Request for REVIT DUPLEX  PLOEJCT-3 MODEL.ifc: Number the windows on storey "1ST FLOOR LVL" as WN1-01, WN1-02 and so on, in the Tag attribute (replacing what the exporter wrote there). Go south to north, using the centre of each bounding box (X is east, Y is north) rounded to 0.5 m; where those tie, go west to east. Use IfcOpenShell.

First a look at what the model holds.

```python
import ifcopenshell
import ifcopenshell.util.element
import ifcopenshell.util.placement

model = ifcopenshell.open("REVIT DUPLEX  PLOEJCT-3 MODEL.ifc")
print(model.schema)
storey = next(s for s in model.by_type("IfcBuildingStorey") if s.Name == "1ST FLOOR LVL")
windows = [e for e in ifcopenshell.util.element.get_decomposition(storey) if e.is_a("IfcWindow")]
for e in sorted(windows, key=lambda e: e.id()):
    origin = ifcopenshell.util.placement.get_local_placement(e.ObjectPlacement)[:3, 3]
    print(e.id(), e.Tag, e.Name, origin.round(2) + 0.0, sep=" | ")
```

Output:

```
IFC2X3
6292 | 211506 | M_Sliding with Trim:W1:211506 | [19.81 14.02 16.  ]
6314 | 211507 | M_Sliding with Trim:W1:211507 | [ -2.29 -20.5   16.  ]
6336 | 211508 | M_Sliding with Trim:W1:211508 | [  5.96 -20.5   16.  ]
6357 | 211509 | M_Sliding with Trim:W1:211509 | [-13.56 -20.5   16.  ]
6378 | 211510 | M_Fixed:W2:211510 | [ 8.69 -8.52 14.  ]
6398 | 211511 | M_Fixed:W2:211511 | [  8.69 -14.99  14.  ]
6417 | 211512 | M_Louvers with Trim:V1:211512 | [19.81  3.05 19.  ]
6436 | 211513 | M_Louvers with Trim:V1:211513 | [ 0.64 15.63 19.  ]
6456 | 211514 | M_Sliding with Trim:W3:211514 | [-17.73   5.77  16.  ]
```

```python
import ifcopenshell
import ifcopenshell.geom
import ifcopenshell.util.element
import ifcopenshell.util.shape

model = ifcopenshell.open("REVIT DUPLEX  PLOEJCT-3 MODEL.ifc")
settings = ifcopenshell.geom.settings()
settings.set("use-world-coords", True)


def centre(element):
    shape = ifcopenshell.geom.create_shape(settings, element)
    return ifcopenshell.util.shape.get_bbox_centroid(shape.geometry)


storey = next(s for s in model.by_type("IfcBuildingStorey") if s.Name == "1ST FLOOR LVL")
windows = [e for e in ifcopenshell.util.element.get_decomposition(storey) if e.is_a("IfcWindow")]

# Insertion points can sit at a corner or the storey origin, so sort by the geometry (in metres).
centres = {e: centre(e) for e in windows}
windows.sort(key=lambda e: (round(centres[e][1] / 0.5), centres[e][0]))

for i, e in enumerate(windows, start=1):
    number = f"WN1-{i:02d}"
    e.Tag = number
    print(e.id(), number)

model.write("REVIT DUPLEX  PLOEJCT-3 MODEL_rev.ifc")
```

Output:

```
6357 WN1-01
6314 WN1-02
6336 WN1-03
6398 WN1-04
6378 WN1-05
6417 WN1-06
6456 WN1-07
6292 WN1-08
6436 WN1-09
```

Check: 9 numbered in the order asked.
